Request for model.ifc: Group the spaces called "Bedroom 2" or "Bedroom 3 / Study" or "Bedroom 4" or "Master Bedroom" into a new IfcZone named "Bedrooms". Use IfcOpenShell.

First a look at what the model holds.

```python
import ifcopenshell

model = ifcopenshell.open("model.ifc")
print(model.schema)
seen = {}
for space in model.by_type("IfcSpace"):
    seen[space.LongName] = seen.get(space.LongName, 0) + 1
for name, count in sorted(seen.items(), key=str):
    print(count, "x", name)
print("zones:", [z.Name for z in model.by_type("IfcZone")][:20])
```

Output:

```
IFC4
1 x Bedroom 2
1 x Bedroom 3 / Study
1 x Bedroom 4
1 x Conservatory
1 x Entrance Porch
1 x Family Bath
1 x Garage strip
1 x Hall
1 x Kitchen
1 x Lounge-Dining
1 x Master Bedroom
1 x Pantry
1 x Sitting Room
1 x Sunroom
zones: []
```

```python
import ifcopenshell
import ifcopenshell.api.group
import ifcopenshell.api.root

model = ifcopenshell.open("model.ifc")

names = {"Bedroom 2", "Bedroom 3 / Study", "Bedroom 4", "Master Bedroom"}
spaces = [s for s in model.by_type("IfcSpace") if s.LongName in names]

zone = ifcopenshell.api.root.create_entity(model, ifc_class="IfcZone", name="Bedrooms")
ifcopenshell.api.group.assign_group(model, products=spaces, group=zone)
print(len(spaces), "spaces in", zone.Name)

model.write("model_updated.ifc")
```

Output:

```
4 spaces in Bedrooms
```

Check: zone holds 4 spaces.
